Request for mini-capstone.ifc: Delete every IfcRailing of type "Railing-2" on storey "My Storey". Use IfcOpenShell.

First a look at what the model holds.

```python
import ifcopenshell
import ifcopenshell.util.element

model = ifcopenshell.open("mini-capstone.ifc")
print(model.schema)
storey = next(s for s in model.by_type("IfcBuildingStorey") if s.Name == "My Storey")
railings = [e for e in ifcopenshell.util.element.get_decomposition(storey) if e.is_a("IfcRailing")]
seen = {}
for e in railings:
    element_type = ifcopenshell.util.element.get_type(e)
    name = element_type.Name if element_type not in (None, e) else None
    seen[name] = seen.get(name, 0) + 1
for name, count in sorted(seen.items(), key=str):
    print(count, "x", name)
```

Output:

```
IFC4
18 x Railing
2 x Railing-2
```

```python
import ifcopenshell
import ifcopenshell.api.root
import ifcopenshell.util.element

model = ifcopenshell.open("mini-capstone.ifc")

storey = next(s for s in model.by_type("IfcBuildingStorey") if s.Name == "My Storey")
railings = [e for e in ifcopenshell.util.element.get_decomposition(storey) if e.is_a("IfcRailing")]
targets = [e for e in railings if (t := ifcopenshell.util.element.get_type(e)) not in (None, e) and t.Name == "Railing-2"]

for e in targets:
    ifcopenshell.api.root.remove_product(model, product=e)
print(len(targets), "removed")

model.write("mini-capstone_v2.ifc")
```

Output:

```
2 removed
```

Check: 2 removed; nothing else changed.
